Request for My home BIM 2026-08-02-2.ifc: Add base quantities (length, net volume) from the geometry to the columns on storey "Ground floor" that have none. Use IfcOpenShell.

First a look at what the model holds.

```python
import ifcopenshell
import ifcopenshell.util.element
import ifcopenshell.util.unit

model = ifcopenshell.open("My home BIM 2026-08-02-2.ifc")
print(model.schema)
for unit_type in ("LENGTHUNIT", "AREAUNIT", "VOLUMEUNIT"):
    print(unit_type, ifcopenshell.util.unit.calculate_unit_scale(model, unit_type))
storey = next(s for s in model.by_type("IfcBuildingStorey") if s.Name == "Ground floor")
columns = [e for e in ifcopenshell.util.element.get_decomposition(storey) if e.is_a("IfcColumn")]
for e in sorted(columns, key=lambda e: e.id()):
    print(e.id(), e.is_a(), e.Name, list(ifcopenshell.util.element.get_psets(e, qtos_only=True)), sep=" | ")
```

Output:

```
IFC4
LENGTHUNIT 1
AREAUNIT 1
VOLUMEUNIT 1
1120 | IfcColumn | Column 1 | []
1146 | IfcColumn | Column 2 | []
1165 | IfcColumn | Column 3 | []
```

```python
import ifcopenshell
import ifcopenshell.api.pset
import ifcopenshell.geom
import ifcopenshell.util.element
import ifcopenshell.util.shape
import ifcopenshell.util.unit

model = ifcopenshell.open("My home BIM 2026-08-02-2.ifc")
unit_scale = ifcopenshell.util.unit.calculate_unit_scale(model)
volume_scale = ifcopenshell.util.unit.calculate_unit_scale(model, "VOLUMEUNIT")
settings = ifcopenshell.geom.settings()

storey = next(s for s in model.by_type("IfcBuildingStorey") if s.Name == "Ground floor")
columns = [e for e in ifcopenshell.util.element.get_decomposition(storey) if e.is_a("IfcColumn")]

for e in sorted(columns, key=lambda e: e.id()):
    if ifcopenshell.util.element.get_psets(e, qtos_only=True, should_inherit=False):
        continue
    # Geometry comes back in metres, in the element's own axes.
    shape = ifcopenshell.geom.create_shape(settings, e)
    values = {
        "Length": ifcopenshell.util.shape.get_z(shape.geometry) / unit_scale,
        "NetVolume": ifcopenshell.util.shape.get_volume(shape.geometry) / volume_scale,
    }
    qto = ifcopenshell.api.pset.add_qto(model, product=e, name="Qto_ColumnBaseQuantities")
    ifcopenshell.api.pset.edit_qto(model, qto=qto, properties=values)
    print(e.id(), {k: round(v, 3) for k, v in values.items()})

model.write("My home BIM 2026-08-02-2-out.ifc")
```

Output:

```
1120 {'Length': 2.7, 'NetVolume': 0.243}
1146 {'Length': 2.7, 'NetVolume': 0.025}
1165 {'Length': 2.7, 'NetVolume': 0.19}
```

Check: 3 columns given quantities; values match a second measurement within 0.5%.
